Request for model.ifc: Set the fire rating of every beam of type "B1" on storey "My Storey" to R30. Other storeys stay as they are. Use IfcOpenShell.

First a look at what the model holds.

```python
import ifcopenshell
import ifcopenshell.util.element

model = ifcopenshell.open("model.ifc")
print(model.schema)
storey = next(s for s in model.by_type("IfcBuildingStorey") if s.Name == "My Storey")
beams = [e for e in ifcopenshell.util.element.get_decomposition(storey) if e.is_a("IfcBeam")]
seen = {}
for e in beams:
    element_type = ifcopenshell.util.element.get_type(e)
    key = (element_type.Name if element_type != e and element_type else None, ifcopenshell.util.element.get_pset(e, "Pset_BeamCommon", "FireRating"))
    seen[key] = seen.get(key, 0) + 1
for (name, value), count in sorted(seen.items(), key=str):
    print(count, "x", name, "|", value)
```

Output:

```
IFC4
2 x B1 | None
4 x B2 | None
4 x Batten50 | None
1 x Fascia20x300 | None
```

```python
import ifcopenshell
import ifcopenshell.api.pset
import ifcopenshell.util.element

model = ifcopenshell.open("model.ifc")

storey = next(s for s in model.by_type("IfcBuildingStorey") if s.Name == "My Storey")
beams = [e for e in ifcopenshell.util.element.get_decomposition(storey) if e.is_a("IfcBeam")]

count = 0
for e in beams:
    element_type = ifcopenshell.util.element.get_type(e)
    if element_type in (None, e) or element_type.Name != "B1":
        continue
    # add_pset returns the element's existing set when there is one.
    pset = ifcopenshell.api.pset.add_pset(model, product=e, name="Pset_BeamCommon")
    ifcopenshell.api.pset.edit_pset(model, pset=pset, properties={"FireRating": "R30"})
    count += 1

print(count, "beams updated")

model.write("model_updated.ifc")
```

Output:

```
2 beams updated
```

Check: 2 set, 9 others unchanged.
